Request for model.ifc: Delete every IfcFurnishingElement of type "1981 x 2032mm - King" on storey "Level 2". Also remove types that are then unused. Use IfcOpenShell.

First a look at what the model holds.

```python
import ifcopenshell
import ifcopenshell.util.element

model = ifcopenshell.open("model.ifc")
print(model.schema)
storey = next(s for s in model.by_type("IfcBuildingStorey") if s.Name == "Level 2")
furniture = [e for e in ifcopenshell.util.element.get_decomposition(storey) if e.is_a("IfcFurnishingElement")]
seen = {}
for e in furniture:
    element_type = ifcopenshell.util.element.get_type(e)
    name = element_type.Name if element_type not in (None, e) else None
    seen[name] = seen.get(name, 0) + 1
for name, count in sorted(seen.items(), key=str):
    print(count, "x", name)
```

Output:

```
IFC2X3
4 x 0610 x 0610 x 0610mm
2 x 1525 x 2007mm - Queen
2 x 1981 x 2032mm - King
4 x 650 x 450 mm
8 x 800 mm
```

```python
import ifcopenshell
import ifcopenshell.api.root
import ifcopenshell.util.element

model = ifcopenshell.open("model.ifc")

storey = next(s for s in model.by_type("IfcBuildingStorey") if s.Name == "Level 2")
furniture = [e for e in ifcopenshell.util.element.get_decomposition(storey) if e.is_a("IfcFurnishingElement")]
targets = [e for e in furniture if (t := ifcopenshell.util.element.get_type(e)) not in (None, e) and t.Name == "1981 x 2032mm - King"]
types = {ifcopenshell.util.element.get_type(e) for e in targets} - {None, *targets}

for e in targets:
    ifcopenshell.api.root.remove_product(model, product=e)
print(len(targets), "removed")

unused = [t for t in types if not ifcopenshell.util.element.get_types(t)]
for t in unused:
    ifcopenshell.api.root.remove_product(model, product=t)
print(len(unused), "unused types removed")

model.write("model_updated.ifc")
```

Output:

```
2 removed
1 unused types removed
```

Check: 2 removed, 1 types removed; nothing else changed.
